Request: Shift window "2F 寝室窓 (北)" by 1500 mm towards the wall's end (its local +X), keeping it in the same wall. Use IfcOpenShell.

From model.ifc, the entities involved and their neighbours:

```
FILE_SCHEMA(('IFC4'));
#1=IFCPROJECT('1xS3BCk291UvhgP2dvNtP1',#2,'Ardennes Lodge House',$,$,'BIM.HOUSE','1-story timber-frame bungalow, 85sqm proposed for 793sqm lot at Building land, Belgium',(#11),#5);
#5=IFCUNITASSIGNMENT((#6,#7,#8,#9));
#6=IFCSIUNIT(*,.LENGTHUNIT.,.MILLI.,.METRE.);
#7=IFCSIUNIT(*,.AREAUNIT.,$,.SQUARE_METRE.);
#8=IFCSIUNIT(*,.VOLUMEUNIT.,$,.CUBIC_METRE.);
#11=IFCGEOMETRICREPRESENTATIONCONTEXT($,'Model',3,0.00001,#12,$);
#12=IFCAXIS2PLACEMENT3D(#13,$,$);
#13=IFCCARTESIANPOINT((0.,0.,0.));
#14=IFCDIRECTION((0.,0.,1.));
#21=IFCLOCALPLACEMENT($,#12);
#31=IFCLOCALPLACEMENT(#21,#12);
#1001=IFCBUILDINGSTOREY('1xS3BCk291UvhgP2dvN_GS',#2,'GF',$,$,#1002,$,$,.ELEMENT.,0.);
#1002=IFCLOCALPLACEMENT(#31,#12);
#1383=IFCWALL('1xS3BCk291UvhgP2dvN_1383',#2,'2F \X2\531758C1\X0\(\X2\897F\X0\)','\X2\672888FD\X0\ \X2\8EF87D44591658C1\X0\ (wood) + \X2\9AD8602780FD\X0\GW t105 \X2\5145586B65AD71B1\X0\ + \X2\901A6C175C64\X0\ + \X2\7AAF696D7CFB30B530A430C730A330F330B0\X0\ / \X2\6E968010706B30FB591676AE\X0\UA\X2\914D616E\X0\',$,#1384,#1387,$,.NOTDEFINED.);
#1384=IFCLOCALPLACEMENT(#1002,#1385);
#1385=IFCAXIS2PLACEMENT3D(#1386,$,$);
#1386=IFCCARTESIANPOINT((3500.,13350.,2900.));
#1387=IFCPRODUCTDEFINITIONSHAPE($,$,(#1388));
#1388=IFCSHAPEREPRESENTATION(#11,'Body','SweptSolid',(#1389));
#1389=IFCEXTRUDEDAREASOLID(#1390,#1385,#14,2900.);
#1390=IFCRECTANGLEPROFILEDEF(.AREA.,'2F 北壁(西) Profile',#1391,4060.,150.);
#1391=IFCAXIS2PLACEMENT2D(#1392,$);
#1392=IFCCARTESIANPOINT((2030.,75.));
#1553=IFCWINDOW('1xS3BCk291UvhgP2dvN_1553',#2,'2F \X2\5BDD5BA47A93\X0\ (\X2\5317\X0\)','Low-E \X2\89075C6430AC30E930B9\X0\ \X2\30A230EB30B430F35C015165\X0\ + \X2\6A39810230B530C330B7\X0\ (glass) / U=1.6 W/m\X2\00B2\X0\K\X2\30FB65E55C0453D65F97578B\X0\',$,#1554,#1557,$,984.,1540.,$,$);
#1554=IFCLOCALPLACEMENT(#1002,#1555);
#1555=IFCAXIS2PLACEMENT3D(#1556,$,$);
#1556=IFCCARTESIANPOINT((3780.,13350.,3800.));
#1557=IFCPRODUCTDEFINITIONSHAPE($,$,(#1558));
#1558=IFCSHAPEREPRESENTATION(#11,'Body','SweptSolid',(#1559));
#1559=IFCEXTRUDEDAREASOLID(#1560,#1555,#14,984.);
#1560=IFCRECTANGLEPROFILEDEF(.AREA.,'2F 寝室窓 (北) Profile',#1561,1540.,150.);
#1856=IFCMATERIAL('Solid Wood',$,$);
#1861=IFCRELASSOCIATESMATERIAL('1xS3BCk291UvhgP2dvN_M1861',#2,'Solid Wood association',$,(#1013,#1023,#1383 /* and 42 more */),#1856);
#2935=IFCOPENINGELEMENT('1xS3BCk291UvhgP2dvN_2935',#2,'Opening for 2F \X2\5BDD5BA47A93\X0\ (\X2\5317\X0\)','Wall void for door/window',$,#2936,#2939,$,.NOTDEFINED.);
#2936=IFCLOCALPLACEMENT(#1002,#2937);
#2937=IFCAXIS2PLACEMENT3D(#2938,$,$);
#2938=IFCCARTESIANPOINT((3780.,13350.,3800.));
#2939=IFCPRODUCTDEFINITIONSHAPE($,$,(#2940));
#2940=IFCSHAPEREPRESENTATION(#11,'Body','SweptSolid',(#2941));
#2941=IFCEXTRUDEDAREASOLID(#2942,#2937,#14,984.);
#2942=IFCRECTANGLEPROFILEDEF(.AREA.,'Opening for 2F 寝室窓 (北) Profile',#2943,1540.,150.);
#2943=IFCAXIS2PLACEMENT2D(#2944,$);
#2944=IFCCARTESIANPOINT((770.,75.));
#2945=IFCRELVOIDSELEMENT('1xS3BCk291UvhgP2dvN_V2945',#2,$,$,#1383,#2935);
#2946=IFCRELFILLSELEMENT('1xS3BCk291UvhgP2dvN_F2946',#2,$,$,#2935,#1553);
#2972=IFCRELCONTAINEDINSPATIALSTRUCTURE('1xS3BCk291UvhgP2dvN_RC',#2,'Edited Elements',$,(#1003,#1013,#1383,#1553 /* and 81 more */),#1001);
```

```python
import ifcopenshell
import ifcopenshell.api.geometry
import ifcopenshell.util.placement

model = ifcopenshell.open("model.ifc")

window = model.by_guid("1xS3BCk291UvhgP2dvN_1553")
opening = window.FillsVoids[0].RelatingOpeningElement
wall = opening.VoidsElements[0].RelatingBuildingElement

wall_matrix = ifcopenshell.util.placement.get_local_placement(wall.ObjectPlacement)
shift = wall_matrix[:3, 0] * 1500.0
before = ifcopenshell.util.placement.get_local_placement(window.ObjectPlacement)[:3, 3].copy()

# The window is not placed relative to its opening, so move both.
for product in (opening, window):
    matrix = ifcopenshell.util.placement.get_local_placement(product.ObjectPlacement)
    matrix[:3, 3] += shift
    ifcopenshell.api.geometry.edit_object_placement(model, product=product, matrix=matrix, is_si=False)

after = ifcopenshell.util.placement.get_local_placement(window.ObjectPlacement)[:3, 3]
print("window moved by", (after - before).round(3) + 0.0)

model.write("model_updated.ifc")
```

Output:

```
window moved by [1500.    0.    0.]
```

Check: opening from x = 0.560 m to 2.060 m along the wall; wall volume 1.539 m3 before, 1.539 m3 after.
